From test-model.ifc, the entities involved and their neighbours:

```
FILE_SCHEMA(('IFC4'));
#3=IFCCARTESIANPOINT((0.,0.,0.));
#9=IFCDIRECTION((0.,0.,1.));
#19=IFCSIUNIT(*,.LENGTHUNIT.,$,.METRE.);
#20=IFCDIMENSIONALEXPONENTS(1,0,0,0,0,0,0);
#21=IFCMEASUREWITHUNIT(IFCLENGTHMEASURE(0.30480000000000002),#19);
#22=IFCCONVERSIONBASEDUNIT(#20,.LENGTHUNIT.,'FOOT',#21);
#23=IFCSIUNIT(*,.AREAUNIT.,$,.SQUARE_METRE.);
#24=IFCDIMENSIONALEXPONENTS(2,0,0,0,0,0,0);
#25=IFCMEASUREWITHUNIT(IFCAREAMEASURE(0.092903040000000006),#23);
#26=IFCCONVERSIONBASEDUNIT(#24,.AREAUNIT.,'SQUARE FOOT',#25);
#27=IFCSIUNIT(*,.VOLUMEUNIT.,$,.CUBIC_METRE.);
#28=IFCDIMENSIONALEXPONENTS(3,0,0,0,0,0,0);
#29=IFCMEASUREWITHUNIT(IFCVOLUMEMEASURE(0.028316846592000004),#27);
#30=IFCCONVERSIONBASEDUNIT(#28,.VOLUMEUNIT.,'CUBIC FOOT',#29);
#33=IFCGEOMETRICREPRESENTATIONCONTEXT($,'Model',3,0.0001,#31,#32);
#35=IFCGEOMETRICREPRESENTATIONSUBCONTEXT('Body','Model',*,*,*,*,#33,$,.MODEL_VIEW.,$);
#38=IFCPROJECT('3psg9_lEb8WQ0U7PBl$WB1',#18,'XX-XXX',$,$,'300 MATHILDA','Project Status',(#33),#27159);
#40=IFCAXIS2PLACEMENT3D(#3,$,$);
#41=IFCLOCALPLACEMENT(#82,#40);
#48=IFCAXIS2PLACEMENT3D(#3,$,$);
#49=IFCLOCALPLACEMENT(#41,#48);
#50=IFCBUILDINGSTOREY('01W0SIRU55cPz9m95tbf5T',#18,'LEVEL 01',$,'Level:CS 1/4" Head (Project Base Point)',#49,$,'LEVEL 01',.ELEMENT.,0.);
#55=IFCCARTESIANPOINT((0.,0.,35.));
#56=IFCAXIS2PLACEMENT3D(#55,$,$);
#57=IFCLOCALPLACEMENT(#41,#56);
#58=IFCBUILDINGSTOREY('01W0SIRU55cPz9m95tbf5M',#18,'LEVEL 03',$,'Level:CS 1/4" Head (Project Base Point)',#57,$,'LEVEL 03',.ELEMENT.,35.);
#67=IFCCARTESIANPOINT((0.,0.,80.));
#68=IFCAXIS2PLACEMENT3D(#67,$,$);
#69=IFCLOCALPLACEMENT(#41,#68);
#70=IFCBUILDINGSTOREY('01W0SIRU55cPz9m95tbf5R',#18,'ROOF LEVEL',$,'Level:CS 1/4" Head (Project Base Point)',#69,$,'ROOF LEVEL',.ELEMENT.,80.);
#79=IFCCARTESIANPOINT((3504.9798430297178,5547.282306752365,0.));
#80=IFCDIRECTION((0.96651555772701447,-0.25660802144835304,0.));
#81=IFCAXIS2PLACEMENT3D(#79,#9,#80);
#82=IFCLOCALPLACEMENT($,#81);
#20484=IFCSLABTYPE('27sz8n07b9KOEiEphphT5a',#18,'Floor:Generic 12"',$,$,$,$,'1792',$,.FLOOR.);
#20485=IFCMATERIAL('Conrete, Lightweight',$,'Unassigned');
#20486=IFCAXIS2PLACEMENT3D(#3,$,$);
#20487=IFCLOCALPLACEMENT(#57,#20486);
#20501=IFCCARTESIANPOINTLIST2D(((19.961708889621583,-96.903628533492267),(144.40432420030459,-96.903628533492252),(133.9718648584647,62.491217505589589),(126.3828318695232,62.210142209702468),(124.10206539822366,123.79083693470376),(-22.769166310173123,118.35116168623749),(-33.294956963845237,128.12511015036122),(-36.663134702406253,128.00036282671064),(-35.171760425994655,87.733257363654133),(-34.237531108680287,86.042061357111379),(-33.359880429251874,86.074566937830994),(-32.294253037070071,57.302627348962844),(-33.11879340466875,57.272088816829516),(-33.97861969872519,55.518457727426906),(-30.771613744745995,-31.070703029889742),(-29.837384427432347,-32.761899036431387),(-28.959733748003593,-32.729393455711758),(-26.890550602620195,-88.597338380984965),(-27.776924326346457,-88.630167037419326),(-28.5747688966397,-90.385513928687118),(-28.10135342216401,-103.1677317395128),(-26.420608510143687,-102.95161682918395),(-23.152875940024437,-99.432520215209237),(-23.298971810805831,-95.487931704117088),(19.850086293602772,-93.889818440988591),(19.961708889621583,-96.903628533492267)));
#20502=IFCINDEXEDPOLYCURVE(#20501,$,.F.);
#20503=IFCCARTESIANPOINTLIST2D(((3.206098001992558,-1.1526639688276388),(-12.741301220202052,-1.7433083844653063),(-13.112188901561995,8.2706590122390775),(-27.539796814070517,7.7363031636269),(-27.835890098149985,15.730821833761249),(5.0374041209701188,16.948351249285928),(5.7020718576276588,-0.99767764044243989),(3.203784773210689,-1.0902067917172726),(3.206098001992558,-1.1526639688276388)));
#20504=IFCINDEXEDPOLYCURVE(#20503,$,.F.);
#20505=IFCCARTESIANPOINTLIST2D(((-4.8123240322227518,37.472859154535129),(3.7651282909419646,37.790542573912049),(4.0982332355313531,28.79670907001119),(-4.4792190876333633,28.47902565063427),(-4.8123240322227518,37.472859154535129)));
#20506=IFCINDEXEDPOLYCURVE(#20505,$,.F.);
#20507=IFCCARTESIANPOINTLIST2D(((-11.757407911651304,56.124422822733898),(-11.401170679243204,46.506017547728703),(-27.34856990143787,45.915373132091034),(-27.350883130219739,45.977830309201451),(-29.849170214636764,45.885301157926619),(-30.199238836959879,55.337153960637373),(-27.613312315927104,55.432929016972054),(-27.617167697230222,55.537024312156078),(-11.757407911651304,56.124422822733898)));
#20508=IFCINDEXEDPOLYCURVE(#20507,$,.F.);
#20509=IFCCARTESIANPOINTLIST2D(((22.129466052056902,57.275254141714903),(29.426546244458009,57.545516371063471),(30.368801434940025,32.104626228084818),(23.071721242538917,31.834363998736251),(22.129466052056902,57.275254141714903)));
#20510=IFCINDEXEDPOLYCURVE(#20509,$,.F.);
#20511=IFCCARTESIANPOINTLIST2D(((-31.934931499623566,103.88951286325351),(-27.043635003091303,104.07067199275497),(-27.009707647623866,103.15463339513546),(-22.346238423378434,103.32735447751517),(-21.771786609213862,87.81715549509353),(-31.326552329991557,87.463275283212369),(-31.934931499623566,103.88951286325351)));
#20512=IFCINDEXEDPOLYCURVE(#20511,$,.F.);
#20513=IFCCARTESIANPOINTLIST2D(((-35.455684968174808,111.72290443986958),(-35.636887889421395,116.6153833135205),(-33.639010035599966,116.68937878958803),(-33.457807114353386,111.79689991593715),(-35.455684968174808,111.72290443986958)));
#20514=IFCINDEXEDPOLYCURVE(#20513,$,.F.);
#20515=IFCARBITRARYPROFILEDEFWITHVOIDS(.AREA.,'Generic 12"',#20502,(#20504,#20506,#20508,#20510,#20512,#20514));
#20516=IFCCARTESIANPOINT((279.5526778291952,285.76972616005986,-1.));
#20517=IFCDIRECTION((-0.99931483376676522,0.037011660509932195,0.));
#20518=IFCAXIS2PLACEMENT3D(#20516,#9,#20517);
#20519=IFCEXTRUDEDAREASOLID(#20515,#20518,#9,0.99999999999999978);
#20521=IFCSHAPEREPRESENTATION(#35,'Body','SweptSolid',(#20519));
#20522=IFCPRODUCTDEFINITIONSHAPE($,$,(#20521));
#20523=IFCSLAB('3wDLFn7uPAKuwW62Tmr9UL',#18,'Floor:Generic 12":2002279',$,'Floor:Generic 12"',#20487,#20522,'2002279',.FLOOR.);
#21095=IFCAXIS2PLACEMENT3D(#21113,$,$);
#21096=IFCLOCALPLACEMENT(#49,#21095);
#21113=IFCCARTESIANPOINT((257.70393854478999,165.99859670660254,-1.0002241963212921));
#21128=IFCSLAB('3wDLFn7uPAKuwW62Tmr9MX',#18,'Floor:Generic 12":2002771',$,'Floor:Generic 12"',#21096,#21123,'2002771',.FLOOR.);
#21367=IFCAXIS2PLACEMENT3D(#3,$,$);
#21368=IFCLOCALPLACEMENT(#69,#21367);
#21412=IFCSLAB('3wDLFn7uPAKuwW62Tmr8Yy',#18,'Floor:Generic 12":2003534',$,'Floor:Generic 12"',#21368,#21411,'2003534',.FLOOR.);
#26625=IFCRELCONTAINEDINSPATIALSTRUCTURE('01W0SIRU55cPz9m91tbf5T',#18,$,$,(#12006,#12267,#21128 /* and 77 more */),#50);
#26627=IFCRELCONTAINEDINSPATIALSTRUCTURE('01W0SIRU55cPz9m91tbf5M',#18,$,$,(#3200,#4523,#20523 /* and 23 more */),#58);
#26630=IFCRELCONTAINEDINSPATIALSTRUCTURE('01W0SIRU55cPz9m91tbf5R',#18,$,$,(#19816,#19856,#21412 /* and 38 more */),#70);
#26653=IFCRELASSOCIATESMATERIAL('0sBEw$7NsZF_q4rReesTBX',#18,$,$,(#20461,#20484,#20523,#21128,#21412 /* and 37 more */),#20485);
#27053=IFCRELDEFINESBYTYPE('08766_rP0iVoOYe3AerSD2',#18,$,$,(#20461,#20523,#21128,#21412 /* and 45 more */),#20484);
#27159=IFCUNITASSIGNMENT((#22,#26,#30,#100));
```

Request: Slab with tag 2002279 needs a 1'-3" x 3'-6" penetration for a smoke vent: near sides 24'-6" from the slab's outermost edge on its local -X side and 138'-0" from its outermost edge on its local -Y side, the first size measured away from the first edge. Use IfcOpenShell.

```python
import numpy as np
import ifcopenshell
import ifcopenshell.api.feature
import ifcopenshell.api.geometry
import ifcopenshell.api.root
import ifcopenshell.geom
import ifcopenshell.util.placement
import ifcopenshell.util.representation
import ifcopenshell.util.shape
import ifcopenshell.util.unit

model = ifcopenshell.open("test-model.ifc")
unit_scale = ifcopenshell.util.unit.calculate_unit_scale(model)
settings = ifcopenshell.geom.settings()


def volume(element):
    """Net volume in cubic metres, openings subtracted."""
    shape = ifcopenshell.geom.create_shape(settings, element)
    return ifcopenshell.util.shape.get_volume(shape.geometry)


slab = model.by_guid("3wDLFn7uPAKuwW62Tmr9UL")
before = volume(slab)

# Extent in the slab's own axes, in metres. The edges named are its -X and -Y sides.
slab_shape = ifcopenshell.geom.create_shape(settings, slab)
vertices = ifcopenshell.util.shape.get_vertices(slab_shape.geometry)
x_min, y_min, bottom = vertices.min(axis=0)
top = vertices[:, 2].max()

opening = ifcopenshell.api.root.create_entity(model, ifc_class="IfcOpeningElement", name="Smoke vent opening", predefined_type="OPENING")
context = ifcopenshell.util.representation.get_context(model, "Model", "Body", "MODEL_VIEW")
width, depth = 0.381, 1.0668
outline = [(0.0, 0.0), (width, 0.0), (width, depth), (0.0, depth), (0.0, 0.0)]
# Overshoot both faces by 50 mm so the cut is clean.
shape = ifcopenshell.api.geometry.add_slab_representation(
    model, context=context, depth=top - bottom + 0.1, polyline=outline
)
ifcopenshell.api.geometry.assign_representation(model, product=opening, representation=shape)

matrix = ifcopenshell.util.placement.get_local_placement(slab.ObjectPlacement)
matrix[:, 3] = matrix @ np.append(np.array([x_min + 7.4676, y_min + 42.0624, bottom - 0.05]) / unit_scale, 1.0)
ifcopenshell.api.geometry.edit_object_placement(model, product=opening, matrix=matrix, is_si=False)
ifcopenshell.api.feature.add_feature(model, feature=opening, element=slab)

after = volume(slab)

print(f"slab volume {before:.3f} -> {after:.3f} m3")

model.write("test-model_v2.ifc")
```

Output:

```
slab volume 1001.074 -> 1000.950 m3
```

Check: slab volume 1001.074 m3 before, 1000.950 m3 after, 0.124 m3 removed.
